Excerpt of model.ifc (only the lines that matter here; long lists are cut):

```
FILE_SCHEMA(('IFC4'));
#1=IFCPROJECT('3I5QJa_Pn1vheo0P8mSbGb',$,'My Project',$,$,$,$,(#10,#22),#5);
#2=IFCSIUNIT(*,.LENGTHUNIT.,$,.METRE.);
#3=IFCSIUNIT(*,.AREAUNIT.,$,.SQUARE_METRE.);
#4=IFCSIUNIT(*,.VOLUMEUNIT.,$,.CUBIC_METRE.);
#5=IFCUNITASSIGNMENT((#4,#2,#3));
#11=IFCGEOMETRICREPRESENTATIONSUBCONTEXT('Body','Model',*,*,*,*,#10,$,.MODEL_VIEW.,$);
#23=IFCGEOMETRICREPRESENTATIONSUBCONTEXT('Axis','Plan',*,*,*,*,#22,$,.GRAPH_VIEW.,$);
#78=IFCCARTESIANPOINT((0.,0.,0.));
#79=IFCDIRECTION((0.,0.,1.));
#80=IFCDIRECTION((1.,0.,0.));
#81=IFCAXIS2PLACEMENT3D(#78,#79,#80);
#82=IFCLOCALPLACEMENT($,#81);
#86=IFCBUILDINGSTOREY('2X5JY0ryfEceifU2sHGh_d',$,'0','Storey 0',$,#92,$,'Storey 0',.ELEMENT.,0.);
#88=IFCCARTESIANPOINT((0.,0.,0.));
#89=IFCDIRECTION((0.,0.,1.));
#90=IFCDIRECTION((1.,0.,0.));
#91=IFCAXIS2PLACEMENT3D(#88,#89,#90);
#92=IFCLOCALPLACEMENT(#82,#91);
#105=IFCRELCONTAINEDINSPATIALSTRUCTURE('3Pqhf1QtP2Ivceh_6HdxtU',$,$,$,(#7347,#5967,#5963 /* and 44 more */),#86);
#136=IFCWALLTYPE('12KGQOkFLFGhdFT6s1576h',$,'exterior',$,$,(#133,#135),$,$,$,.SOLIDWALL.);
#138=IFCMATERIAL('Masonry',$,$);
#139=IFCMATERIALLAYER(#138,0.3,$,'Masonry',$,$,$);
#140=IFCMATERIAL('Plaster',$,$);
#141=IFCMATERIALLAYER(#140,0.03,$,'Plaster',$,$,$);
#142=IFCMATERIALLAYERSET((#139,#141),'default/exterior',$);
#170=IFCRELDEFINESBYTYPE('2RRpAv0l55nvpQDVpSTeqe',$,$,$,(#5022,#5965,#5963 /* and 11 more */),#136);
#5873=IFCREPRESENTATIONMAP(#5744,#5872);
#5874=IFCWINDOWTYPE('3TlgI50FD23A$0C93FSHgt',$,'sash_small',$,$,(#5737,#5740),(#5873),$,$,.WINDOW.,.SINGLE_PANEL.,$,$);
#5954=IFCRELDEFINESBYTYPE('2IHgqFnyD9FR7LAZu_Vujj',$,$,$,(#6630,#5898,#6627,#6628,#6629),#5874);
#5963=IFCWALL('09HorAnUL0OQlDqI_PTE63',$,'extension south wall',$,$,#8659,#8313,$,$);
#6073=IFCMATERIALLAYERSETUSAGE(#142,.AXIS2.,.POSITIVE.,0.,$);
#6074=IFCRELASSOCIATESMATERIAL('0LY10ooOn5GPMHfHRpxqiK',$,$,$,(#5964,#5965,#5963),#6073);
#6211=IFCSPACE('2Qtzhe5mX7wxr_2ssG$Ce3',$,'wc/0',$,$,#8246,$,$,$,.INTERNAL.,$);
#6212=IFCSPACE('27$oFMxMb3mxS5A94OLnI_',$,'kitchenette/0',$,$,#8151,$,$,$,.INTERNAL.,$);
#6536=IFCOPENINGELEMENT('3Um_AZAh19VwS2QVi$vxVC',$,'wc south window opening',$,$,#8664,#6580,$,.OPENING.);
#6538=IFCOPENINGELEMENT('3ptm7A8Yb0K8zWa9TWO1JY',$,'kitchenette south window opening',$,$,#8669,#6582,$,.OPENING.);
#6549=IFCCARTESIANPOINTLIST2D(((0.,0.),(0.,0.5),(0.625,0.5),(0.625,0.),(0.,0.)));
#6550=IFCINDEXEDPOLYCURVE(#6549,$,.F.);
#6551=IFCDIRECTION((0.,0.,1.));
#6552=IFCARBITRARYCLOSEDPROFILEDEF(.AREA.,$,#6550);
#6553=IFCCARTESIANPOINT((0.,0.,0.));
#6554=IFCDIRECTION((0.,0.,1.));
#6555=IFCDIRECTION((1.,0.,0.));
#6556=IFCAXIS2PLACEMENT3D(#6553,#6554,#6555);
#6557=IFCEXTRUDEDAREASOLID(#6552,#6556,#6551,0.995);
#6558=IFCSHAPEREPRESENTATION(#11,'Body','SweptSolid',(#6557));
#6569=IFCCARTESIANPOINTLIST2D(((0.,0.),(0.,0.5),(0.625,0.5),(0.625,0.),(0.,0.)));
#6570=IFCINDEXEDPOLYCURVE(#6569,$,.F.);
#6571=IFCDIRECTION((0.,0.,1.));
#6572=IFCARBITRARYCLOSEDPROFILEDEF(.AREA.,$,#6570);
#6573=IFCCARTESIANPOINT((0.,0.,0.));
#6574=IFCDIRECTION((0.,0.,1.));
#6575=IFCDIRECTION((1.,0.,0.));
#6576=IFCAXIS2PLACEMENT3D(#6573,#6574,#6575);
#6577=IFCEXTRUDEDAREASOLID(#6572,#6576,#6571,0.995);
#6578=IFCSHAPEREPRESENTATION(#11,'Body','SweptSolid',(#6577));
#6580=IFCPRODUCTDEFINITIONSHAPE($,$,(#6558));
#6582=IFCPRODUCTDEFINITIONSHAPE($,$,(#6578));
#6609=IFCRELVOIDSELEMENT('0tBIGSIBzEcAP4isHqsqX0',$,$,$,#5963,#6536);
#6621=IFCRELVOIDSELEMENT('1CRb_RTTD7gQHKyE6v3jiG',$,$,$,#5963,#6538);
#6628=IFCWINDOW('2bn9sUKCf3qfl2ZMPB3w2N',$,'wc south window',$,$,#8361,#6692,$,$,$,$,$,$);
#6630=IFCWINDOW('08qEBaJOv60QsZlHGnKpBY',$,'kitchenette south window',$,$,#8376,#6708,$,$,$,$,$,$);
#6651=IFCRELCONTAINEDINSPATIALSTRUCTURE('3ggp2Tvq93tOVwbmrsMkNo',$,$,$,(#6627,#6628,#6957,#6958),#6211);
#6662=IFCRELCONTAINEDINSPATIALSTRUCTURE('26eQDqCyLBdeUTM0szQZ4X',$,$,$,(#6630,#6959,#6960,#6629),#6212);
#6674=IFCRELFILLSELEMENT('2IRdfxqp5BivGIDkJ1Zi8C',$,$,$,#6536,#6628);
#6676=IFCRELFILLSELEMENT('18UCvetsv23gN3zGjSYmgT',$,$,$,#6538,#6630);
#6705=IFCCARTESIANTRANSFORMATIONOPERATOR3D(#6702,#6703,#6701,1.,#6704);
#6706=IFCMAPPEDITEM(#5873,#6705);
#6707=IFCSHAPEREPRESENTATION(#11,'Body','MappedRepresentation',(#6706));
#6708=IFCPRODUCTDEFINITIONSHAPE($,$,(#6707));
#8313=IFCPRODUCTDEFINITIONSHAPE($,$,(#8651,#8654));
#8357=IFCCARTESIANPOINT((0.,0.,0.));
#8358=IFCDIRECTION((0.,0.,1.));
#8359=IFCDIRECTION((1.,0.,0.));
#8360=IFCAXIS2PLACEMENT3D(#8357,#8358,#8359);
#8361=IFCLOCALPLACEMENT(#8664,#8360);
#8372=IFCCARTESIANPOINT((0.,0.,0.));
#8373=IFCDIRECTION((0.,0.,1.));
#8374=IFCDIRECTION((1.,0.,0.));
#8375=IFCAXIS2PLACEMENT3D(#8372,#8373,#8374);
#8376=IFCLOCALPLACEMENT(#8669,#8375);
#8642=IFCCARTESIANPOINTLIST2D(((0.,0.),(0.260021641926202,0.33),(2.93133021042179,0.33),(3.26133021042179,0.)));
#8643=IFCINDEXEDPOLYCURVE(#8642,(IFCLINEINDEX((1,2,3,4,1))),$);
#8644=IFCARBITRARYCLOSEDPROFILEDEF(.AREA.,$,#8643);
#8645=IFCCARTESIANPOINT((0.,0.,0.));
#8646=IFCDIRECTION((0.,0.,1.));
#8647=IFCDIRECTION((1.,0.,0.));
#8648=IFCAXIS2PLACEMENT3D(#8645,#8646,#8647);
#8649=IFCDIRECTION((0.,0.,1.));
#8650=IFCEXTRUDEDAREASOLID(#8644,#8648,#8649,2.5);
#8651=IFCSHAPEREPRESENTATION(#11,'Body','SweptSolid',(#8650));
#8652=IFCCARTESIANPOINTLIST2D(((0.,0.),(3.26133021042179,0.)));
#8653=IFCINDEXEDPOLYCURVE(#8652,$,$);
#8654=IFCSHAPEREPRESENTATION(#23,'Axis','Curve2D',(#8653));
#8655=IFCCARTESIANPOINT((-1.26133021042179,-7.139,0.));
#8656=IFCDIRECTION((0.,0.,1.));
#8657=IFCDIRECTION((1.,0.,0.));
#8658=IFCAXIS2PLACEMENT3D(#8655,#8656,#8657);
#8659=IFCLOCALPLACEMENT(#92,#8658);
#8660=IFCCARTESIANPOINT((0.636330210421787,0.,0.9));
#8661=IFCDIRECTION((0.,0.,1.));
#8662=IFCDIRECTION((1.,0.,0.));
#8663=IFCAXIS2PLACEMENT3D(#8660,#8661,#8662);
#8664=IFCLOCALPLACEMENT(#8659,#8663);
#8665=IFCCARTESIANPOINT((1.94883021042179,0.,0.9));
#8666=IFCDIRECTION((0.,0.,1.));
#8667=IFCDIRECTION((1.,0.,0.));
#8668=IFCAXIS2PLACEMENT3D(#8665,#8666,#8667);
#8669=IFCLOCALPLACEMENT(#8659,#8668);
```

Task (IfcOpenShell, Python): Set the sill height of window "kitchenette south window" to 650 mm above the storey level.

```python
import numpy as np
import ifcopenshell
import ifcopenshell.api.geometry
import ifcopenshell.geom
import ifcopenshell.util.element
import ifcopenshell.util.placement
import ifcopenshell.util.shape
import ifcopenshell.util.unit

model = ifcopenshell.open("model.ifc")
unit_scale = ifcopenshell.util.unit.calculate_unit_scale(model)

window = model.by_guid("08qEBaJOv60QsZlHGnKpBY")
opening = window.FillsVoids[0].RelatingOpeningElement
storey = ifcopenshell.util.element.get_container(window, ifc_class="IfcBuildingStorey")
level = ifcopenshell.util.placement.get_local_placement(storey.ObjectPlacement)[2, 3]

# The opening's origin need not be at the sill, so measure its lowest point.
shape = ifcopenshell.geom.create_shape(ifcopenshell.geom.settings(), opening)
bottom = ifcopenshell.util.shape.get_shape_bottom_elevation(shape, shape.geometry) / unit_scale
dz = level + 0.65 - bottom

shift = np.array([0.0, 0.0, dz])
# The window is placed relative to its opening, so it follows when the opening moves.
matrix = ifcopenshell.util.placement.get_local_placement(opening.ObjectPlacement)
matrix[:3, 3] += shift
ifcopenshell.api.geometry.edit_object_placement(
    model, product=opening, matrix=matrix, is_si=False, should_transform_children=True
)

print(f"moved by {dz * unit_scale:+.3f} m")

model.write("model-out.ifc")
```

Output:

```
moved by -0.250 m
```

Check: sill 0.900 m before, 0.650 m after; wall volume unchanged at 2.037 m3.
